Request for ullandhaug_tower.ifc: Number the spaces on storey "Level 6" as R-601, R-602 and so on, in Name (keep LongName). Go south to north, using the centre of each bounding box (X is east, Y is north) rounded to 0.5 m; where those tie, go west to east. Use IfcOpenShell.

First a look at what the model holds.

```python
import ifcopenshell
import ifcopenshell.util.element
import ifcopenshell.util.placement

model = ifcopenshell.open("ullandhaug_tower.ifc")
print(model.schema)
storey = next(s for s in model.by_type("IfcBuildingStorey") if s.Name == "Level 6")
spaces = [e for e in ifcopenshell.util.element.get_decomposition(storey) if e.is_a("IfcSpace")]
for e in sorted(spaces, key=lambda e: e.id()):
    origin = ifcopenshell.util.placement.get_local_placement(e.ObjectPlacement)[:3, 3]
    print(e.id(), e.Name, e.LongName, origin.round(2) + 0.0, sep=" | ")
```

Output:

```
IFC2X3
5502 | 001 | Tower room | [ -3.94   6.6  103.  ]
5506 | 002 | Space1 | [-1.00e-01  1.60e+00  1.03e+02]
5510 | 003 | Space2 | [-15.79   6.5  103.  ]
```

```python
import ifcopenshell
import ifcopenshell.geom
import ifcopenshell.util.element
import ifcopenshell.util.shape

model = ifcopenshell.open("ullandhaug_tower.ifc")
settings = ifcopenshell.geom.settings()
settings.set("use-world-coords", True)


def centre(element):
    shape = ifcopenshell.geom.create_shape(settings, element)
    return ifcopenshell.util.shape.get_bbox_centroid(shape.geometry)


storey = next(s for s in model.by_type("IfcBuildingStorey") if s.Name == "Level 6")
spaces = [e for e in ifcopenshell.util.element.get_decomposition(storey) if e.is_a("IfcSpace")]

# Insertion points can sit at a corner or the storey origin, so sort by the geometry (in metres).
centres = {e: centre(e) for e in spaces}
spaces.sort(key=lambda e: (round(centres[e][1] / 0.5), centres[e][0]))

for i, e in enumerate(spaces, start=1):
    number = f"R-6{i:02d}"
    e.Name = number
    print(e.id(), number)

model.write("ullandhaug_tower_v2.ifc")
```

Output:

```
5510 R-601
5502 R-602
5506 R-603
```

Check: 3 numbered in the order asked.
